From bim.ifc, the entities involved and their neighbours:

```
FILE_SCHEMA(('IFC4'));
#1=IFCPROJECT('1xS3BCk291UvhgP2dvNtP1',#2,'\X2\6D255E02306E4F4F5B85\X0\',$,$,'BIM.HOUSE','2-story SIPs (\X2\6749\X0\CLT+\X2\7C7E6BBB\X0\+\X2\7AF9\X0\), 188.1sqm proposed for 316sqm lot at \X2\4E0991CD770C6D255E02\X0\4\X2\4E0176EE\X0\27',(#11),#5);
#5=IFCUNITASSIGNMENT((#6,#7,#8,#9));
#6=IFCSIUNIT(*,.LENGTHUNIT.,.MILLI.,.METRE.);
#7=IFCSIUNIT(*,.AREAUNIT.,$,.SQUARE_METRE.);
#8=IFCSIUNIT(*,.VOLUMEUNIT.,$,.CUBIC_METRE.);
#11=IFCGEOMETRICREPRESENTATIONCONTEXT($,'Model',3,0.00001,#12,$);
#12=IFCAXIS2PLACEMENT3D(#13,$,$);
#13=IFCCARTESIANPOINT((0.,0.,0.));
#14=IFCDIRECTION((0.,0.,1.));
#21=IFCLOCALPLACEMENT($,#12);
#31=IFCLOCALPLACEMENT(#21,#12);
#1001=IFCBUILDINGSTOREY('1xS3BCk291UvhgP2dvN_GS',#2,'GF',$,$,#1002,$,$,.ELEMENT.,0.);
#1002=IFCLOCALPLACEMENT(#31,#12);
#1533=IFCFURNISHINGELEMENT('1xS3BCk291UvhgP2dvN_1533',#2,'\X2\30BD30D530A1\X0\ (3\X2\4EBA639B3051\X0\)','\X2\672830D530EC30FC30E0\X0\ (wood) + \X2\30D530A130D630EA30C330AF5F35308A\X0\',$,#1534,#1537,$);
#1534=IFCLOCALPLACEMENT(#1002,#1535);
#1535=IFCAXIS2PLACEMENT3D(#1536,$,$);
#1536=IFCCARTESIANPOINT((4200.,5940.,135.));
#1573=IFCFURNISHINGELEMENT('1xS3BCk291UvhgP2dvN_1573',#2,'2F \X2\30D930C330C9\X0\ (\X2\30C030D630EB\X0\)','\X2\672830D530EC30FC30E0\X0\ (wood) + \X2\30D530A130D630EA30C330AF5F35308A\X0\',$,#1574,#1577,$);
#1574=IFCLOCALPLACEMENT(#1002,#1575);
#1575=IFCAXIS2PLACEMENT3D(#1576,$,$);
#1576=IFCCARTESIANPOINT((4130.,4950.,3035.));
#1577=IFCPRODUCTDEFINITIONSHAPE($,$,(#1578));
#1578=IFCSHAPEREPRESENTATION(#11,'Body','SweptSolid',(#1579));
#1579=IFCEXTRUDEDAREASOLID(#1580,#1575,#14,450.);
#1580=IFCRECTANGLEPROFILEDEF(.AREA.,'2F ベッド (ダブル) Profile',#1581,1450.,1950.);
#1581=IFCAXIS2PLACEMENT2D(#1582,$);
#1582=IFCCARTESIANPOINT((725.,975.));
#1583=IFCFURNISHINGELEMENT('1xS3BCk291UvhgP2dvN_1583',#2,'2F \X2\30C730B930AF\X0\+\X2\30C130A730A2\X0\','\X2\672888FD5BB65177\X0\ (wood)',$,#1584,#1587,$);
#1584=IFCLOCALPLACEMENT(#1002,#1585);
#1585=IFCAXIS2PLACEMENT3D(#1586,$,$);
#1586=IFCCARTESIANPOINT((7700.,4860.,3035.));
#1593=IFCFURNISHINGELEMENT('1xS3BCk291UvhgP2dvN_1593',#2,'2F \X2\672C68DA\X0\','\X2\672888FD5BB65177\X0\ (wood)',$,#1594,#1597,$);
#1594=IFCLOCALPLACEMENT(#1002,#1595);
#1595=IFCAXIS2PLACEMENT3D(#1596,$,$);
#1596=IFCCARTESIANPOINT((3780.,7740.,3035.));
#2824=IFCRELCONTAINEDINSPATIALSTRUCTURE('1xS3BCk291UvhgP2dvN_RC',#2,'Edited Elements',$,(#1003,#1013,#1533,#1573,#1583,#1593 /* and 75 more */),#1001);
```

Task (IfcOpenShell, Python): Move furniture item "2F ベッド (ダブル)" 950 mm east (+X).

```python
import ifcopenshell
import ifcopenshell.api.geometry
import ifcopenshell.util.placement
import ifcopenshell.util.unit

model = ifcopenshell.open("bim.ifc")
unit_scale = ifcopenshell.util.unit.calculate_unit_scale(model)

item = model.by_guid("1xS3BCk291UvhgP2dvN_1573")
matrix = ifcopenshell.util.placement.get_local_placement(item.ObjectPlacement)
matrix[0, 3] += 0.95 / unit_scale
ifcopenshell.api.geometry.edit_object_placement(model, product=item, matrix=matrix, is_si=False)

print(ifcopenshell.util.placement.get_local_placement(item.ObjectPlacement).round(3) + 0.0)

model.write("bim_rev.ifc")
```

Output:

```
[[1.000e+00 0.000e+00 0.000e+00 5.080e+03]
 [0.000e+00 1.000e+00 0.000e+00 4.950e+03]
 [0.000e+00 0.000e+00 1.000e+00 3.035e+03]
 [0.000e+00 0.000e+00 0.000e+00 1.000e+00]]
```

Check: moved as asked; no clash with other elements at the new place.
